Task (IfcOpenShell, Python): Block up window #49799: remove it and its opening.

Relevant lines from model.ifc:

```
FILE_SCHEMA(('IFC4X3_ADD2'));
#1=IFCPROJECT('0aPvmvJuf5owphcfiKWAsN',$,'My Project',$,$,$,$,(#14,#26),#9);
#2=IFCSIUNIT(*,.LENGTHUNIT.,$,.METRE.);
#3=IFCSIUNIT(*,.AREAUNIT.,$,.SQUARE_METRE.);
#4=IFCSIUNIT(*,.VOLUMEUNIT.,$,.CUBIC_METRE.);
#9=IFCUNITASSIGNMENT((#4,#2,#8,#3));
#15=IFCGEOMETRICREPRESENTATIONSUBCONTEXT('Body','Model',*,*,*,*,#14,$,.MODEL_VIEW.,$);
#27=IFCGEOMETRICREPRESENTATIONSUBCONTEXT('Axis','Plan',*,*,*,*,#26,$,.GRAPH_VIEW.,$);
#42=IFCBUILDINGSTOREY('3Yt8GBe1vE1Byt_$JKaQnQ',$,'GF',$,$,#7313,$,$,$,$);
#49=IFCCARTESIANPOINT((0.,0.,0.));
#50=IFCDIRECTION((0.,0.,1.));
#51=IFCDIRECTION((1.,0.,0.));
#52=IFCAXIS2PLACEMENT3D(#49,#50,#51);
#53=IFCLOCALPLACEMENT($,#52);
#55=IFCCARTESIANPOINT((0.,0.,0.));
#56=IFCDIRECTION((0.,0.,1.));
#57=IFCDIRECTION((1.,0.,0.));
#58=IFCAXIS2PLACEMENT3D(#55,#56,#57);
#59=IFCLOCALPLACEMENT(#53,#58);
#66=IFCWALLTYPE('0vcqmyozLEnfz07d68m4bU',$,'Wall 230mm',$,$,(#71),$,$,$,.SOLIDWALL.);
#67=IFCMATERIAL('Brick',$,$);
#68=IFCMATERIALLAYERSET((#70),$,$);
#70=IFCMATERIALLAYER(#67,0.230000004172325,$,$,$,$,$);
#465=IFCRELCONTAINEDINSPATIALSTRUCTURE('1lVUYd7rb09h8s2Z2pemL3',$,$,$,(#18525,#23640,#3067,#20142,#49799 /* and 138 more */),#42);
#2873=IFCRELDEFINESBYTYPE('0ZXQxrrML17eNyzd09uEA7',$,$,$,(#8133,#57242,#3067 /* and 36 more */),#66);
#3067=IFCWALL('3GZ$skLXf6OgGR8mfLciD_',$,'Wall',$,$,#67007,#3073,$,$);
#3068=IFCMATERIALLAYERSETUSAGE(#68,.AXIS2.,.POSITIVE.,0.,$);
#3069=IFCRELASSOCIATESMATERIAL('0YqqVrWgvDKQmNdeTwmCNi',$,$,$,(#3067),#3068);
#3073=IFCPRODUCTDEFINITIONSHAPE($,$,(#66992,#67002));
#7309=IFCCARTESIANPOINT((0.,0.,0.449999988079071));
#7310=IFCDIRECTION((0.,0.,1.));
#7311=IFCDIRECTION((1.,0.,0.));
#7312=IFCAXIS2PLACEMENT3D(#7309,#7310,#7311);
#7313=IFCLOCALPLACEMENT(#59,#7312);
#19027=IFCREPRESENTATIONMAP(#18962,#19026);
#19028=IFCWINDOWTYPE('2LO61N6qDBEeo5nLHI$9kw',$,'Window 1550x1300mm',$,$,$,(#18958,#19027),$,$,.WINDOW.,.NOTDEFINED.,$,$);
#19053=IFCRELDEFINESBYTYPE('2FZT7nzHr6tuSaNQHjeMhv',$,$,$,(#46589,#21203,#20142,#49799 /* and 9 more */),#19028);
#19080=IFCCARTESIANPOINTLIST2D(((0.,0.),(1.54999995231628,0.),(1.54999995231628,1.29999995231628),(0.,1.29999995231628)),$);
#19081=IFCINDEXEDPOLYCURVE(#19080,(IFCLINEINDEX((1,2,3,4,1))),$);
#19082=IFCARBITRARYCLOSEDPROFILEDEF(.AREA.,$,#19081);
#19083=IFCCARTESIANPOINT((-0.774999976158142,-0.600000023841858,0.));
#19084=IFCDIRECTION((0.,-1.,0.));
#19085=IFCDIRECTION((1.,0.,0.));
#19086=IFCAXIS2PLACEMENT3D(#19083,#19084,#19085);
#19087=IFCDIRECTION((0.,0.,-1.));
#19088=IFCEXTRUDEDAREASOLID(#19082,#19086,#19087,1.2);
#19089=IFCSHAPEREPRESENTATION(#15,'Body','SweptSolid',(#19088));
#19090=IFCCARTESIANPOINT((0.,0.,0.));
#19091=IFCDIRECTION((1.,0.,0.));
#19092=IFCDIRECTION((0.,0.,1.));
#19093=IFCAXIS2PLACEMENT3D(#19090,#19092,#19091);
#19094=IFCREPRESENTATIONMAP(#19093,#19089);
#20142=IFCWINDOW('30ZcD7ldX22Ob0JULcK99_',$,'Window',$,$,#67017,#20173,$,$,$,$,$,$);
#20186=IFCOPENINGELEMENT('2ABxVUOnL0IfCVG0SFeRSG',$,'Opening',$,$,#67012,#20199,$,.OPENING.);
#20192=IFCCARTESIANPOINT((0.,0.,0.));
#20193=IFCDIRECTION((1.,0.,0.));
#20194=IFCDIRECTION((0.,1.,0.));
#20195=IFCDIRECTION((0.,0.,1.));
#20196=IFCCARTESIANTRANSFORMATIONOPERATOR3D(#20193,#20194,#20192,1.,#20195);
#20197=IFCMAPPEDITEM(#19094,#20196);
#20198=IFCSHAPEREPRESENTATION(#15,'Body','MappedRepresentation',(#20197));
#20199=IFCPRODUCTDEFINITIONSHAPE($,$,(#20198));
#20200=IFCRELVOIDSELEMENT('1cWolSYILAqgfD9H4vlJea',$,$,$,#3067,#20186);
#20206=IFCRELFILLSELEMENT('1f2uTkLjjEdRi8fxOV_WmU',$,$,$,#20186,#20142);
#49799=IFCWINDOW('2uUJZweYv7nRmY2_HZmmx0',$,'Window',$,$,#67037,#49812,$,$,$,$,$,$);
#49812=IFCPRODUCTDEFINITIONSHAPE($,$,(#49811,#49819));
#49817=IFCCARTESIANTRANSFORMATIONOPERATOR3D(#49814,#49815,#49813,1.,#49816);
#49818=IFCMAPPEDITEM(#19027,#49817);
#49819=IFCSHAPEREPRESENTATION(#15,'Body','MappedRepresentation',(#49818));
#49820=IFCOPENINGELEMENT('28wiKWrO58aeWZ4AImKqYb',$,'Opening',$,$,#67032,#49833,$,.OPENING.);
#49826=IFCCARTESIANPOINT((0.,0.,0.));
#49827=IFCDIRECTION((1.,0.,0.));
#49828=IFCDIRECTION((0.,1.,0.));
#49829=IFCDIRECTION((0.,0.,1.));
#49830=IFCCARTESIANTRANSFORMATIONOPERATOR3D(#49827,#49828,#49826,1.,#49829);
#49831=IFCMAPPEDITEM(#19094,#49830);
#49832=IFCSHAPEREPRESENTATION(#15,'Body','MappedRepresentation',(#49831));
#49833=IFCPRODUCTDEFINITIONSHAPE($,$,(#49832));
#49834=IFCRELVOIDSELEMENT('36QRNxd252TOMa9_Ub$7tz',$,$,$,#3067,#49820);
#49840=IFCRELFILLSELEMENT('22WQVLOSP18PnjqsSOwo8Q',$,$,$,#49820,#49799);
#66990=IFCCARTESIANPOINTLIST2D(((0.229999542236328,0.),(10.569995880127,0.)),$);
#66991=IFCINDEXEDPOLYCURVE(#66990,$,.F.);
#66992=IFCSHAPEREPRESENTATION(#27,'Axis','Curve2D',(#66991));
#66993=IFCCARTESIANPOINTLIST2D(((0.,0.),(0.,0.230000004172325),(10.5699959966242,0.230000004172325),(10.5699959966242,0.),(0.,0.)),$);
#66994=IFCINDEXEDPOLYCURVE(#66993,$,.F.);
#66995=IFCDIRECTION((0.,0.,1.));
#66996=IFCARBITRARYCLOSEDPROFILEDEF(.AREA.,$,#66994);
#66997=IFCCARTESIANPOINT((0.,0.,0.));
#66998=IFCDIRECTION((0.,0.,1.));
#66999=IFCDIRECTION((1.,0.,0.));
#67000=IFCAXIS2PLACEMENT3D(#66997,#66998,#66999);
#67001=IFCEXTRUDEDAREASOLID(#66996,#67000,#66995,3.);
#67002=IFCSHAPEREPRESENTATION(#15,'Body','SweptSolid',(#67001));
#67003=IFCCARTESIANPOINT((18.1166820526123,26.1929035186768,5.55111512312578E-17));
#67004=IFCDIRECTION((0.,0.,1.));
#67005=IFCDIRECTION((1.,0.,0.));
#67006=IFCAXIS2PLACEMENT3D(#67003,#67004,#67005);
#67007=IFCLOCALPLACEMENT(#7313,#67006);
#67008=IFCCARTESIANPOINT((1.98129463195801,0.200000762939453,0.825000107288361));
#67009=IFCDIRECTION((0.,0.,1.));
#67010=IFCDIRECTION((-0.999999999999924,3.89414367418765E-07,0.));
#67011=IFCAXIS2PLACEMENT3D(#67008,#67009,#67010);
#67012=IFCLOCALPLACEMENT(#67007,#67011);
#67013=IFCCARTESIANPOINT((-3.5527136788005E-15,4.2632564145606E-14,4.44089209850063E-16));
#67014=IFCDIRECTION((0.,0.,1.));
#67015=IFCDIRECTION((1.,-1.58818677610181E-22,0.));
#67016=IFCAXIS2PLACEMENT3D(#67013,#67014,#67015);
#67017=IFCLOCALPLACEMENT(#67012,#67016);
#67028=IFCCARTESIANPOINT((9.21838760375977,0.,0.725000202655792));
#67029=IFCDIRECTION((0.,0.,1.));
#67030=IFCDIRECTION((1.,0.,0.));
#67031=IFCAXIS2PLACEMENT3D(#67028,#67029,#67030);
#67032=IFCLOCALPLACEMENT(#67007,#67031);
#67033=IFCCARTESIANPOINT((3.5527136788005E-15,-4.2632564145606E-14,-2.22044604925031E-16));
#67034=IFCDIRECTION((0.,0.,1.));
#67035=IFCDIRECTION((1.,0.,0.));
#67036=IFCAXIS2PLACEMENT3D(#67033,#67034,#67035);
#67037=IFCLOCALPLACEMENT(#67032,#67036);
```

```python
import ifcopenshell
import ifcopenshell.api.feature
import ifcopenshell.api.root
import ifcopenshell.geom
import ifcopenshell.util.shape

model = ifcopenshell.open("model.ifc")
settings = ifcopenshell.geom.settings()


def volume(element):
    """Net volume in cubic metres, openings subtracted."""
    shape = ifcopenshell.geom.create_shape(settings, element)
    return ifcopenshell.util.shape.get_volume(shape.geometry)


window = model.by_id(49799)
opening = window.FillsVoids[0].RelatingOpeningElement
wall = opening.VoidsElements[0].RelatingBuildingElement
before = volume(wall)

ifcopenshell.api.root.remove_product(model, product=window)
ifcopenshell.api.feature.remove_feature(model, feature=opening)

after = volume(wall)

print(f"wall volume {before:.3f} -> {after:.3f} m3")

model.write("model-out.ifc")
```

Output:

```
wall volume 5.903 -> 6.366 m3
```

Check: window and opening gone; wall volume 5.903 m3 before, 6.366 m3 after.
